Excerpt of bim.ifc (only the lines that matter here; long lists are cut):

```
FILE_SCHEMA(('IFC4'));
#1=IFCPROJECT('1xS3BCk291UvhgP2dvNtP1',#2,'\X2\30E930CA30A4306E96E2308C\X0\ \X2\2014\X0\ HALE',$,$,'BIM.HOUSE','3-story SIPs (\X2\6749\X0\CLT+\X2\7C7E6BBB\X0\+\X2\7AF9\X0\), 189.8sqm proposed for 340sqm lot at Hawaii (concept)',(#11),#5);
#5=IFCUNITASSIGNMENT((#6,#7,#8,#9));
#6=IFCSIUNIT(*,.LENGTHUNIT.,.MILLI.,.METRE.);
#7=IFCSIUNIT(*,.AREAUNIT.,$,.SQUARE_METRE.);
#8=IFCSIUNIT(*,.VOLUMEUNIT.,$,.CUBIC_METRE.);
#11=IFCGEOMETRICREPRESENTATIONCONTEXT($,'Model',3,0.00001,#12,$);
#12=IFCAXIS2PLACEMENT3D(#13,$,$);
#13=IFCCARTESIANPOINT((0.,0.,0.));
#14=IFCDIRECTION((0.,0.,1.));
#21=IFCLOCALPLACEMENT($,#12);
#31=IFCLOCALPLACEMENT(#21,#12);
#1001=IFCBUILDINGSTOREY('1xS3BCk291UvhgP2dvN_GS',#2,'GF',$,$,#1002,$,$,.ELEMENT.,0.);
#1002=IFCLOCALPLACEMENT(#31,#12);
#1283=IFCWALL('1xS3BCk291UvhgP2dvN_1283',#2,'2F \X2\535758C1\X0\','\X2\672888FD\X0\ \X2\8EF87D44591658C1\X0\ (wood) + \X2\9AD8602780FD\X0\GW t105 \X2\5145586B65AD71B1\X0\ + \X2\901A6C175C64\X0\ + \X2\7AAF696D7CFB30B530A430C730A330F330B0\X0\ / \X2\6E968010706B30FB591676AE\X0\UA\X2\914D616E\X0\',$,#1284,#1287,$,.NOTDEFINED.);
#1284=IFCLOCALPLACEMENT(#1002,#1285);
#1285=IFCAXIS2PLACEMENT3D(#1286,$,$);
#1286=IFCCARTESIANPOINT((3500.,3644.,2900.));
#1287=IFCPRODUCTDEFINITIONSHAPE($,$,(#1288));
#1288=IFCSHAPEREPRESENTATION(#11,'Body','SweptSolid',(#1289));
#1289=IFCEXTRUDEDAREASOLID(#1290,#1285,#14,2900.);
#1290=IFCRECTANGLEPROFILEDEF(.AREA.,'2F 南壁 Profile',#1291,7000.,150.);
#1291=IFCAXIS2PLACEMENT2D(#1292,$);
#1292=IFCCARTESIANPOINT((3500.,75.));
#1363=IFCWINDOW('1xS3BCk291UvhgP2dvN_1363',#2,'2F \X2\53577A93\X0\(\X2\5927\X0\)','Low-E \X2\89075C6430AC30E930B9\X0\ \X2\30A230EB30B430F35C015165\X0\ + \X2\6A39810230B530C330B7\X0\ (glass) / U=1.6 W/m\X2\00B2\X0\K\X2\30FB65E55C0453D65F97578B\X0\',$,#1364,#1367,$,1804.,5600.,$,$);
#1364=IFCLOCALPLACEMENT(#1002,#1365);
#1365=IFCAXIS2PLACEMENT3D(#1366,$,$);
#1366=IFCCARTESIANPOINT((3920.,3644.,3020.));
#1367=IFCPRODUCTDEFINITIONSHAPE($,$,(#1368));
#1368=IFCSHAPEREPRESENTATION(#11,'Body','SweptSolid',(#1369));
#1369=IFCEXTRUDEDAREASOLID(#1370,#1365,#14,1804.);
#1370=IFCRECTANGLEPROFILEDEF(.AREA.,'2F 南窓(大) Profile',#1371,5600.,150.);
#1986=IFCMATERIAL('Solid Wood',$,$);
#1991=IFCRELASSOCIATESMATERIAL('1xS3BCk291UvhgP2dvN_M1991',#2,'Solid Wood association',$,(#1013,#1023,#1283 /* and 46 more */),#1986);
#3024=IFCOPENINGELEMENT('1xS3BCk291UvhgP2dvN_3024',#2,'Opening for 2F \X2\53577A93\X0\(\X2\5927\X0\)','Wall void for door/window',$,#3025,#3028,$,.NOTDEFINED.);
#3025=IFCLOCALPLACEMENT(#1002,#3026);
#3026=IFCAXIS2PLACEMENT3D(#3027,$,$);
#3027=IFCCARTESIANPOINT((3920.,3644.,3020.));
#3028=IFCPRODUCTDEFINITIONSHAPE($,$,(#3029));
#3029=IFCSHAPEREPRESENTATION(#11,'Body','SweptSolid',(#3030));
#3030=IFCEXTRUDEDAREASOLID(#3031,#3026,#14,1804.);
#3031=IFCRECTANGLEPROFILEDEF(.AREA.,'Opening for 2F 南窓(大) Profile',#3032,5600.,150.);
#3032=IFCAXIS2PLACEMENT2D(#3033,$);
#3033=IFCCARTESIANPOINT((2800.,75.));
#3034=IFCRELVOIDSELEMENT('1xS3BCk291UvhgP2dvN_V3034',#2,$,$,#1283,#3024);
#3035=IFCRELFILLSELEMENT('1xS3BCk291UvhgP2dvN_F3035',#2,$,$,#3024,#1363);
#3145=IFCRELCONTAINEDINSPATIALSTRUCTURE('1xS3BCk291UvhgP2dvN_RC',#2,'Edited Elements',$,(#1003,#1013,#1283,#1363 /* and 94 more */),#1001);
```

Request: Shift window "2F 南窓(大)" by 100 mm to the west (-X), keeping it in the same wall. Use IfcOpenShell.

```python
import ifcopenshell
import ifcopenshell.api.geometry
import ifcopenshell.util.placement
import ifcopenshell.util.unit

model = ifcopenshell.open("bim.ifc")
unit_scale = ifcopenshell.util.unit.calculate_unit_scale(model)

window = model.by_guid("1xS3BCk291UvhgP2dvN_1363")
opening = window.FillsVoids[0].RelatingOpeningElement
wall = opening.VoidsElements[0].RelatingBuildingElement

wall_matrix = ifcopenshell.util.placement.get_local_placement(wall.ObjectPlacement)
shift = wall_matrix[:3, 0] * -0.1 / unit_scale
before = ifcopenshell.util.placement.get_local_placement(window.ObjectPlacement)[:3, 3].copy()

# The window is not placed relative to its opening, so move both.
for product in (opening, window):
    matrix = ifcopenshell.util.placement.get_local_placement(product.ObjectPlacement)
    matrix[:3, 3] += shift
    ifcopenshell.api.geometry.edit_object_placement(model, product=product, matrix=matrix, is_si=False)

after = ifcopenshell.util.placement.get_local_placement(window.ObjectPlacement)[:3, 3]
print("window moved by", (after - before).round(3) + 0.0)

model.write("bim_updated.ifc")
```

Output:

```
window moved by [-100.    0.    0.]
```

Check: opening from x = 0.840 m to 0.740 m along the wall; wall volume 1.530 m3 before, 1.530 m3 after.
